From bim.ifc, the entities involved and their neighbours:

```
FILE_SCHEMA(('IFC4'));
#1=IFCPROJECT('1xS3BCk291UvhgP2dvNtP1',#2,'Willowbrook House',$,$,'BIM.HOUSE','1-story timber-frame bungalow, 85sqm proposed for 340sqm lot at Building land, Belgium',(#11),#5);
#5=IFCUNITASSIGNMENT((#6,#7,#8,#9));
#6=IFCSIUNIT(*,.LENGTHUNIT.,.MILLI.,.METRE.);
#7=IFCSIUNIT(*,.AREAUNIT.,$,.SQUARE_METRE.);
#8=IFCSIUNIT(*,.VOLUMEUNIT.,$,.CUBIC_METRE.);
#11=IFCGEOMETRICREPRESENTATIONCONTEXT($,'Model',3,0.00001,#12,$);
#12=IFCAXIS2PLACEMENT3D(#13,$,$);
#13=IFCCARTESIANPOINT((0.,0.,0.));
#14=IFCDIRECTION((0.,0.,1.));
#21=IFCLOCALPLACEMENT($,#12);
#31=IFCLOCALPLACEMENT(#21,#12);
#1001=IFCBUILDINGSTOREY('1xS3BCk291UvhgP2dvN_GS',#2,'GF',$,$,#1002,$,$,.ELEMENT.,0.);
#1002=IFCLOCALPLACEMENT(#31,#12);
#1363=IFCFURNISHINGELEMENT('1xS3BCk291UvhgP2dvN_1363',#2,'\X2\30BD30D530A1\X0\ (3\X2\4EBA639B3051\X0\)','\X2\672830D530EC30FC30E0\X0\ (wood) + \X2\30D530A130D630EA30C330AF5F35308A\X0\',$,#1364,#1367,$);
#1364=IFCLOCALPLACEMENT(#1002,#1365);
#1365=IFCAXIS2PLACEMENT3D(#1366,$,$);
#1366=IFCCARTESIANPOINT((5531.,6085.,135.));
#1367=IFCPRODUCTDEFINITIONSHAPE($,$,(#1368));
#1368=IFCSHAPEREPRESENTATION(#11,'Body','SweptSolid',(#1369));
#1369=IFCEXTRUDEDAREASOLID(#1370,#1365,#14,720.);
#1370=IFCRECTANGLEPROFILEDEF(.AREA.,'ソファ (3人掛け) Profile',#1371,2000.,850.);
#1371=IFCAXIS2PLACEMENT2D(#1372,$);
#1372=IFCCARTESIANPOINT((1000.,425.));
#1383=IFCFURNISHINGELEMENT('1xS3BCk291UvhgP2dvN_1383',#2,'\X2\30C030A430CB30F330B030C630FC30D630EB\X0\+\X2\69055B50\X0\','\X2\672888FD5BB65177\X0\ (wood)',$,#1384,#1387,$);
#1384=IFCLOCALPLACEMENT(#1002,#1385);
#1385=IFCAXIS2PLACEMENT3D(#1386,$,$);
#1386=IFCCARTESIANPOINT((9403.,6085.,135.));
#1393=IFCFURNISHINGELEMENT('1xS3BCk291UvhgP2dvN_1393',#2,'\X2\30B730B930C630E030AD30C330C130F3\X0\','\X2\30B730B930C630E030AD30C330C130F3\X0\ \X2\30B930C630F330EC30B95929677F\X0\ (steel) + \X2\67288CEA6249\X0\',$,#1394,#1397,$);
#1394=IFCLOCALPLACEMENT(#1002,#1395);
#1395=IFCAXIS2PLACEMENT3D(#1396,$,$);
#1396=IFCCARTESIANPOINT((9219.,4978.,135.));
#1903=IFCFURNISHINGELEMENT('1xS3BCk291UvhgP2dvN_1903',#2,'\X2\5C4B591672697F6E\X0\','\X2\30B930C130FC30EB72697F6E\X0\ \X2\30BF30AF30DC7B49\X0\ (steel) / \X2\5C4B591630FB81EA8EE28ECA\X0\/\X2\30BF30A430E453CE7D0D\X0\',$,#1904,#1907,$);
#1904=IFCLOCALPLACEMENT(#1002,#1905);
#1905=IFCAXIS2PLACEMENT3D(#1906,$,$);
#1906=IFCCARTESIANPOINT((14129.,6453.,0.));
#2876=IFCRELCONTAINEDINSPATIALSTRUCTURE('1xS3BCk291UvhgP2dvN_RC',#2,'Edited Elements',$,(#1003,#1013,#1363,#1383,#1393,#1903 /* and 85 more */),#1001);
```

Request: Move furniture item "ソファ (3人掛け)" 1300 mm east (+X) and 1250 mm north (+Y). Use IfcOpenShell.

```python
import ifcopenshell
import ifcopenshell.api.geometry
import ifcopenshell.util.placement

model = ifcopenshell.open("bim.ifc")

item = model.by_guid("1xS3BCk291UvhgP2dvN_1363")
matrix = ifcopenshell.util.placement.get_local_placement(item.ObjectPlacement)
matrix[0, 3] += 1300.0
matrix[1, 3] += 1250.0
ifcopenshell.api.geometry.edit_object_placement(model, product=item, matrix=matrix, is_si=False)

print(ifcopenshell.util.placement.get_local_placement(item.ObjectPlacement).round(3) + 0.0)

model.write("bim_edited.ifc")
```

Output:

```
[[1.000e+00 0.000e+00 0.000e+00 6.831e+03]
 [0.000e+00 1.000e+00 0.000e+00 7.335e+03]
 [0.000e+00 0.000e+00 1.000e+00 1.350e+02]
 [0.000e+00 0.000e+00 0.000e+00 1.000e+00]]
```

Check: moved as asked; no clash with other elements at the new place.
